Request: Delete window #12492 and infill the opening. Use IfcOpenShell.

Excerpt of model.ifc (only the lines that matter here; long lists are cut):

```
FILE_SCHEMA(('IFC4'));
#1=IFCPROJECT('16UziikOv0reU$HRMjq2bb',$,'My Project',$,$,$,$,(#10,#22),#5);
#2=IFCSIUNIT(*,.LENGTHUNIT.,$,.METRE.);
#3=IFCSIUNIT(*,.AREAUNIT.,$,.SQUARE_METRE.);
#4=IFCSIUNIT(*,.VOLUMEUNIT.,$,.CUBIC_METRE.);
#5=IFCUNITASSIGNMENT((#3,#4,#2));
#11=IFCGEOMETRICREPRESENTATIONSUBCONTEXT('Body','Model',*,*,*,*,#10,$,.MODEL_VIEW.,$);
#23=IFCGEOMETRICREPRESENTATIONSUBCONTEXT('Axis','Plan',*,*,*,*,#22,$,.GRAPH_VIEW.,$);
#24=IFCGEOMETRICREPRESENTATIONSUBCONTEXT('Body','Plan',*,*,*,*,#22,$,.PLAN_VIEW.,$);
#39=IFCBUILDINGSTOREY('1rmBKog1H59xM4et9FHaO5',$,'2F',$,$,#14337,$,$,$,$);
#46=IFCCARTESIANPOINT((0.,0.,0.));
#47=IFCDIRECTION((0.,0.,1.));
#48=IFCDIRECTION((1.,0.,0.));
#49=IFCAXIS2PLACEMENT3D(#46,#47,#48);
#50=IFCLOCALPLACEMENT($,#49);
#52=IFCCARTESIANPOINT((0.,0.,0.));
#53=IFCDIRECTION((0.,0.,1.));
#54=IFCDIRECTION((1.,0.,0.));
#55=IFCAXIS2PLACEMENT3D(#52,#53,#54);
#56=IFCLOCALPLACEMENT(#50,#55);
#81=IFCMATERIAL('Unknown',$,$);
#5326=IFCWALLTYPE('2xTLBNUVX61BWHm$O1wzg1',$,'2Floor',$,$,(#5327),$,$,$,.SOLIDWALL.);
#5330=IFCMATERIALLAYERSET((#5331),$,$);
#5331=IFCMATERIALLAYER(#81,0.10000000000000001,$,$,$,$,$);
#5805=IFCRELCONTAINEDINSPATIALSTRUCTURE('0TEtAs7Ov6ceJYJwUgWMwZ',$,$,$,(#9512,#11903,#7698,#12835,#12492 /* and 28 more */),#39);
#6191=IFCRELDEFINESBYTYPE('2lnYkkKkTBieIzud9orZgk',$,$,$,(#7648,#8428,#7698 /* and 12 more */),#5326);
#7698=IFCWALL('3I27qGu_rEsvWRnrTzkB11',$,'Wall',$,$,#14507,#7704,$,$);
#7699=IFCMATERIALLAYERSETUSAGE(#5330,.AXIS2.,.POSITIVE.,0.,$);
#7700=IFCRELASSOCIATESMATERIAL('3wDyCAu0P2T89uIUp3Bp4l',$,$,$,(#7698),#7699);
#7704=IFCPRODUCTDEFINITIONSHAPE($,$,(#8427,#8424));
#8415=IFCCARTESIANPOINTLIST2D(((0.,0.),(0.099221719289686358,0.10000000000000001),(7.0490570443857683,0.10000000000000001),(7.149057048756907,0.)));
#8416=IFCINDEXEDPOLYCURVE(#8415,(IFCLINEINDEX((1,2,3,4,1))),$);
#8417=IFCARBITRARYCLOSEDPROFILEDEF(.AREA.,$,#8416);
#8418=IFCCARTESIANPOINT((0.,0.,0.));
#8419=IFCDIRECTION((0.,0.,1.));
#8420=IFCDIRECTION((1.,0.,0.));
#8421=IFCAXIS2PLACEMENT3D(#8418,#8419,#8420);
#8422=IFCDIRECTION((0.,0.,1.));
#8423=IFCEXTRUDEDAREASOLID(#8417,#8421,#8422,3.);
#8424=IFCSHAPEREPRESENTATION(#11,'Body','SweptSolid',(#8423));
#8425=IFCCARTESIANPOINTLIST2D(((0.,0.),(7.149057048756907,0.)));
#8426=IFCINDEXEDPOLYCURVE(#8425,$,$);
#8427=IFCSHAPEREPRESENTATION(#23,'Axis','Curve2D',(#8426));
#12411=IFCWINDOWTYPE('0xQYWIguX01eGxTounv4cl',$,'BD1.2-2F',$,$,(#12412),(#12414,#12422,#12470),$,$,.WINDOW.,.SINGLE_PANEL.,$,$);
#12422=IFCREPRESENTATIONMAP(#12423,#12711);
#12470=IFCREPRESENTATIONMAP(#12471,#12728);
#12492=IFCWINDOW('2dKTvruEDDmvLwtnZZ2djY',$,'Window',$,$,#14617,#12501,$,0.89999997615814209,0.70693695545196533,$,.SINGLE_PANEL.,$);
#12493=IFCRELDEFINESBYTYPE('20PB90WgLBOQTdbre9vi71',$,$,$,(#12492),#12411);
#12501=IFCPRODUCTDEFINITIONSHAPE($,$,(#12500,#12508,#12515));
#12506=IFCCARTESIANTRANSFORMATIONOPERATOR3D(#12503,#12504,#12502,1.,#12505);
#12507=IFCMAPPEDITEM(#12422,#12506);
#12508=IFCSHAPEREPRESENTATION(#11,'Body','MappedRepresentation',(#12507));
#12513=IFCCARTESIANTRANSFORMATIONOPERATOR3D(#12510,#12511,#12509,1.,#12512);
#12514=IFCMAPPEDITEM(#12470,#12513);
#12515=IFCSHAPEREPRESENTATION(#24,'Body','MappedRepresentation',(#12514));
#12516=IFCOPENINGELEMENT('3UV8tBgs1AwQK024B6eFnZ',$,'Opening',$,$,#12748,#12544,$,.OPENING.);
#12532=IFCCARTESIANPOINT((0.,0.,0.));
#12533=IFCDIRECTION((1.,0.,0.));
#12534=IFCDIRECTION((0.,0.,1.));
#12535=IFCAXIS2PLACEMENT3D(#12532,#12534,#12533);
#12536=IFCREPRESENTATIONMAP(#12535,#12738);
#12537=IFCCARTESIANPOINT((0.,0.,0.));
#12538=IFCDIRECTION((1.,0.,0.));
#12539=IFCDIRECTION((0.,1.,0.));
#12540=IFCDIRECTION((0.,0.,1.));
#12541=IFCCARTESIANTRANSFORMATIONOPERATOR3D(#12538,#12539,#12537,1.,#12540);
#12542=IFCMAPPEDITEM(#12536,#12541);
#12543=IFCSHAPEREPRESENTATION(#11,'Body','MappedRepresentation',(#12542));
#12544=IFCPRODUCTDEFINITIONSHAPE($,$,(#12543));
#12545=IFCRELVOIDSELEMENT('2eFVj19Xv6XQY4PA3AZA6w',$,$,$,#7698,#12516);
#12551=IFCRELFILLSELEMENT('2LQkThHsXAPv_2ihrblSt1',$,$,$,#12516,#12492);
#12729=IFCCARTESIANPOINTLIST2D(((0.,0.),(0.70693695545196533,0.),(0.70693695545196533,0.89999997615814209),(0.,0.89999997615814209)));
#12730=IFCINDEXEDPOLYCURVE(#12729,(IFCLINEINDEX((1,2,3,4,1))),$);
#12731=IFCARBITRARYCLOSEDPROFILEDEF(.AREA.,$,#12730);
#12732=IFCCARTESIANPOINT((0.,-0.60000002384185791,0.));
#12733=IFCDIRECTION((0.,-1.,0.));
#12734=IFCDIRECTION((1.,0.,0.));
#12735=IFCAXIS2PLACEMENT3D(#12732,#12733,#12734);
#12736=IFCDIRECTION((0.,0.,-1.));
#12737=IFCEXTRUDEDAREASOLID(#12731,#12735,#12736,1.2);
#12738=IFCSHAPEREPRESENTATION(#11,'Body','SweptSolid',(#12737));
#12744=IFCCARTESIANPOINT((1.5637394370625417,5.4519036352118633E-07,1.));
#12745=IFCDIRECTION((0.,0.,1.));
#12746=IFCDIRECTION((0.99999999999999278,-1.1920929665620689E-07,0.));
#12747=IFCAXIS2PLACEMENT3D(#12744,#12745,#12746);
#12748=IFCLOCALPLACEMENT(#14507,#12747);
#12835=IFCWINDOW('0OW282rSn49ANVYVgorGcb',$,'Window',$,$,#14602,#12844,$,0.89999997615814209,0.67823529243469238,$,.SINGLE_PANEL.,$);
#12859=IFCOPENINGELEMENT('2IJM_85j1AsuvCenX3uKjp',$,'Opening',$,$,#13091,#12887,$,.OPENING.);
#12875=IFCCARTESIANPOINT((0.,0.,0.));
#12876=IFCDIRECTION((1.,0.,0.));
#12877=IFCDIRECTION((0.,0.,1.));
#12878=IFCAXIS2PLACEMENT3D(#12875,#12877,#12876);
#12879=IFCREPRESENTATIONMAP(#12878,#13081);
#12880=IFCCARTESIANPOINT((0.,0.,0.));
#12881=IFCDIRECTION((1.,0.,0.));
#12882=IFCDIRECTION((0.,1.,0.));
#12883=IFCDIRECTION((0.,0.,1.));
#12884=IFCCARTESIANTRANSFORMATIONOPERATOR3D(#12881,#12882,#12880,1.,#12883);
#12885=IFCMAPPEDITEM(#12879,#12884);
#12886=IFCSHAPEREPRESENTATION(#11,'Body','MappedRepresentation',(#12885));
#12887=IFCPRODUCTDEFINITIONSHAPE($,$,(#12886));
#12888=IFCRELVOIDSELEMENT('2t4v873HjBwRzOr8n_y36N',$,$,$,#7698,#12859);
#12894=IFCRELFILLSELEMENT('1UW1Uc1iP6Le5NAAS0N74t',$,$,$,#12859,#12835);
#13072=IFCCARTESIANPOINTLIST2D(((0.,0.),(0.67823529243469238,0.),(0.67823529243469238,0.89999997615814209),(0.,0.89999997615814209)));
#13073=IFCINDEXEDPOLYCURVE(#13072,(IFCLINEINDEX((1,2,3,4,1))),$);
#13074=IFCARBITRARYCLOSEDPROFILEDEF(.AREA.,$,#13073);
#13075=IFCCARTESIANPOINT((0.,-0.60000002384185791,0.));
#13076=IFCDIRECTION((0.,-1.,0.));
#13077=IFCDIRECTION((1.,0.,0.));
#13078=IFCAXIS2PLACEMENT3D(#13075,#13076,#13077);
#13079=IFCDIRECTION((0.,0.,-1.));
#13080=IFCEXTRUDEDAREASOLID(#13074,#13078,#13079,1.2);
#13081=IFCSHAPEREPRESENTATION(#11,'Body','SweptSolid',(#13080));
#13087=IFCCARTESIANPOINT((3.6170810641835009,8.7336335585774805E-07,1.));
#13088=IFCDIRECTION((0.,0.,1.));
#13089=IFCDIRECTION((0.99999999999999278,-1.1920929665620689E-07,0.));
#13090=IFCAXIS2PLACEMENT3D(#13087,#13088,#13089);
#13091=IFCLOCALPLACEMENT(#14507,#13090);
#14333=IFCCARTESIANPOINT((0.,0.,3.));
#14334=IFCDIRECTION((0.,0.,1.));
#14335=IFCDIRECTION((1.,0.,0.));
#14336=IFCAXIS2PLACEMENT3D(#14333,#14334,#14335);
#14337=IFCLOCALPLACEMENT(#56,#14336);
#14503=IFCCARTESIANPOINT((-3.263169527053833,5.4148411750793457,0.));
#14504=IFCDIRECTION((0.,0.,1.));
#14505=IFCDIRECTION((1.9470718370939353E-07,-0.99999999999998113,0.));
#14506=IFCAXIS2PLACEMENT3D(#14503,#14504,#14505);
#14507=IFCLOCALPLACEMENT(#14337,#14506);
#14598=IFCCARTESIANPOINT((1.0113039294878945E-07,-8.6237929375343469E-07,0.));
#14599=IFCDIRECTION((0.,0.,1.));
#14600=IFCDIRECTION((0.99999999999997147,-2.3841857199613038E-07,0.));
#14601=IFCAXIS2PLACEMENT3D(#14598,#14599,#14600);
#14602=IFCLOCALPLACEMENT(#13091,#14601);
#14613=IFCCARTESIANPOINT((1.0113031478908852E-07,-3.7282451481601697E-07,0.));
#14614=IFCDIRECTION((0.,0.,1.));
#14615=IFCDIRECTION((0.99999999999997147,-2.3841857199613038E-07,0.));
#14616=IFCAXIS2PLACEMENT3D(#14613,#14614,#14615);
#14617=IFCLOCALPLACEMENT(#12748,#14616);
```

```python
import ifcopenshell
import ifcopenshell.api.feature
import ifcopenshell.api.root
import ifcopenshell.geom
import ifcopenshell.util.shape

model = ifcopenshell.open("model.ifc")
settings = ifcopenshell.geom.settings()


def volume(element):
    """Net volume in cubic metres, openings subtracted."""
    shape = ifcopenshell.geom.create_shape(settings, element)
    return ifcopenshell.util.shape.get_volume(shape.geometry)


window = model.by_guid("2dKTvruEDDmvLwtnZZ2djY")
opening = window.FillsVoids[0].RelatingOpeningElement
wall = opening.VoidsElements[0].RelatingBuildingElement
before = volume(wall)

ifcopenshell.api.root.remove_product(model, product=window)
ifcopenshell.api.feature.remove_feature(model, feature=opening)

after = volume(wall)

print(f"wall volume {before:.3f} -> {after:.3f} m3")

model.write("model-out.ifc")
```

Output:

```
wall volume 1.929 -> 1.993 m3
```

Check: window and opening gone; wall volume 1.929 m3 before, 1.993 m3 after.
